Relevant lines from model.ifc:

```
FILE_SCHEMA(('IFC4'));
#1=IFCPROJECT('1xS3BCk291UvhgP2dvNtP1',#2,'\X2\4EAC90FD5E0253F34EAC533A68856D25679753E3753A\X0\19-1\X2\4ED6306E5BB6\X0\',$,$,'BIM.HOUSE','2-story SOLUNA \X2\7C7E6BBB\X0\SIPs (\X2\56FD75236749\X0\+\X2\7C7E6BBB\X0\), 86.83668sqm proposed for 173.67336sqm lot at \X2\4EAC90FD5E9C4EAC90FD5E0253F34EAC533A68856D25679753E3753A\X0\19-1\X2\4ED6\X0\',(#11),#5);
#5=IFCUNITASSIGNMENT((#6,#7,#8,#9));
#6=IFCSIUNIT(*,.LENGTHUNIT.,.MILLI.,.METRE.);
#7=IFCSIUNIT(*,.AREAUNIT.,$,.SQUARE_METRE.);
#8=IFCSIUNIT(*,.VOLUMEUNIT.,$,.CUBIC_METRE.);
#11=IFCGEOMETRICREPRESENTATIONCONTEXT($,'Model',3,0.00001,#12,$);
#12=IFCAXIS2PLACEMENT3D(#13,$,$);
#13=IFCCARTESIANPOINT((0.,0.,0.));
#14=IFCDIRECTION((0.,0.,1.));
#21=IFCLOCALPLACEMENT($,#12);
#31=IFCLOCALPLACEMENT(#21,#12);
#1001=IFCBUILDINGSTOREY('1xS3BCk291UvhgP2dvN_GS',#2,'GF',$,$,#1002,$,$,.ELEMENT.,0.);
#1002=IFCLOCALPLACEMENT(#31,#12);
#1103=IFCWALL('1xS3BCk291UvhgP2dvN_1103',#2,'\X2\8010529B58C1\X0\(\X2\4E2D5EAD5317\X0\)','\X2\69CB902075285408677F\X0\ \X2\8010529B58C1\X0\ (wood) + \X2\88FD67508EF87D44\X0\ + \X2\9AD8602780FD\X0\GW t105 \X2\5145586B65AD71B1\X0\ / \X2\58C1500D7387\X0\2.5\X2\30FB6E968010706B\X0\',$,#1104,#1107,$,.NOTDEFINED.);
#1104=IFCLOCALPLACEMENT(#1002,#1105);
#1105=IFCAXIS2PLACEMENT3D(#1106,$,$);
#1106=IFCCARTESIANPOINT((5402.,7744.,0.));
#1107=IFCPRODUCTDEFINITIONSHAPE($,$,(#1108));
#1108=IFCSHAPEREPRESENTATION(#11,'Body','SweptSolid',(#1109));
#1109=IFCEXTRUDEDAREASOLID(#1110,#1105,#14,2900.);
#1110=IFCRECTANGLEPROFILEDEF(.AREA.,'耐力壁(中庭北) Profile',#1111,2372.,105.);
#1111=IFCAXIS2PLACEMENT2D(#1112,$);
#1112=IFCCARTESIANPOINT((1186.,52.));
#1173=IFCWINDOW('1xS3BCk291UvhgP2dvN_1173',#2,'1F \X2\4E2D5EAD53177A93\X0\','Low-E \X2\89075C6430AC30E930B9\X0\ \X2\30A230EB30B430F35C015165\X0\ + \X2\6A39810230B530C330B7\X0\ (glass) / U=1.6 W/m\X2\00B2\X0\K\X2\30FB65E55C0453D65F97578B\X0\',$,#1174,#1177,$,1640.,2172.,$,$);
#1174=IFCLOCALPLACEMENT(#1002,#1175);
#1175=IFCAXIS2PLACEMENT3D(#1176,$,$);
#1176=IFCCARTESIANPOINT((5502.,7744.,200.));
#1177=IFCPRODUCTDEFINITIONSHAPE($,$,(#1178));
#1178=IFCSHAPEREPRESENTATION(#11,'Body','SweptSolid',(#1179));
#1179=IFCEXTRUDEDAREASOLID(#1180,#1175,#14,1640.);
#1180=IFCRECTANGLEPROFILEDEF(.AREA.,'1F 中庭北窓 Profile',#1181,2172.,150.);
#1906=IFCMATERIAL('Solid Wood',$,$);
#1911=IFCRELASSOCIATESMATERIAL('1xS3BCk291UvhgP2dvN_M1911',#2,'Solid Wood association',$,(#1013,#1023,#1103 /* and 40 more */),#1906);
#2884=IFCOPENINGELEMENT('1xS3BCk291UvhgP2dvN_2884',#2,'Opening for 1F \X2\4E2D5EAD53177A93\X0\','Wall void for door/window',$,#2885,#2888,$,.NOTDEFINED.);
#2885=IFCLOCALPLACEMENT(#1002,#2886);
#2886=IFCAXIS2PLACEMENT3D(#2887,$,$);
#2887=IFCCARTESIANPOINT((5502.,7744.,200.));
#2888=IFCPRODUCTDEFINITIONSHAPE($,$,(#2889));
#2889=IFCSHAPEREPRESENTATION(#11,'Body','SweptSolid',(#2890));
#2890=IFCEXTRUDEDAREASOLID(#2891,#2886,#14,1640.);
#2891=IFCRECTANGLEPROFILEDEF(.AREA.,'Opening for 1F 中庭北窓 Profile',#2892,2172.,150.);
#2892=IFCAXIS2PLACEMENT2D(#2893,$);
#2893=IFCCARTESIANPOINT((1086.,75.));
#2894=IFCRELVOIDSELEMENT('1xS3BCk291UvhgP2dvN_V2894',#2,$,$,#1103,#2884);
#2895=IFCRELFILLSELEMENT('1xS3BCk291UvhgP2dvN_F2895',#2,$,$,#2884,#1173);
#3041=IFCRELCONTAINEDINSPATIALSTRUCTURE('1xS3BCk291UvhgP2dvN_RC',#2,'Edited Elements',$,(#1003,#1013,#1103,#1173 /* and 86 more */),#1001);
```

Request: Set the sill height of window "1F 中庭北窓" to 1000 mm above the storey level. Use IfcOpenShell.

```python
import numpy as np
import ifcopenshell
import ifcopenshell.api.geometry
import ifcopenshell.geom
import ifcopenshell.util.element
import ifcopenshell.util.placement
import ifcopenshell.util.shape
import ifcopenshell.util.unit

model = ifcopenshell.open("model.ifc")
unit_scale = ifcopenshell.util.unit.calculate_unit_scale(model)

window = model.by_id(1173)
opening = window.FillsVoids[0].RelatingOpeningElement
storey = ifcopenshell.util.element.get_container(window, ifc_class="IfcBuildingStorey")
level = ifcopenshell.util.placement.get_local_placement(storey.ObjectPlacement)[2, 3]

# The opening's origin need not be at the sill, so measure its lowest point.
shape = ifcopenshell.geom.create_shape(ifcopenshell.geom.settings(), opening)
bottom = ifcopenshell.util.shape.get_shape_bottom_elevation(shape, shape.geometry) / unit_scale
dz = level + 1 / unit_scale - bottom

shift = np.array([0.0, 0.0, dz])
# The window is not placed relative to its opening, so move both.
for product in (opening, window):
    matrix = ifcopenshell.util.placement.get_local_placement(product.ObjectPlacement)
    matrix[:3, 3] += shift
    ifcopenshell.api.geometry.edit_object_placement(model, product=product, matrix=matrix, is_si=False)

print(f"moved by {dz * unit_scale:+.3f} m")

model.write("model_updated.ifc")
```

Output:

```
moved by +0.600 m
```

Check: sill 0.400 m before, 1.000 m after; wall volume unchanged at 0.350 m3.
